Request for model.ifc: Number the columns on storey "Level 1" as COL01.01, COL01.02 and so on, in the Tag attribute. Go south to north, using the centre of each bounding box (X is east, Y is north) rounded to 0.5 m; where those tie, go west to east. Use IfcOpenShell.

First a look at what the model holds.

```python
import ifcopenshell
import ifcopenshell.util.element
import ifcopenshell.util.placement

model = ifcopenshell.open("model.ifc")
print(model.schema)
storey = next(s for s in model.by_type("IfcBuildingStorey") if s.Name == "Level 1")
columns = [e for e in ifcopenshell.util.element.get_decomposition(storey) if e.is_a("IfcColumn")]
for e in sorted(columns, key=lambda e: e.id()):
    origin = ifcopenshell.util.placement.get_local_placement(e.ObjectPlacement)[:3, 3]
    print(e.id(), e.Tag, e.Name, origin.round(2) + 0.0, sep=" | ")
```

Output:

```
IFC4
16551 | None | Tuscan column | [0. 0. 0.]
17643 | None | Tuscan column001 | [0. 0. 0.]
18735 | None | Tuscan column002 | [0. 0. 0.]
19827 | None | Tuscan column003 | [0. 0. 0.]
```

```python
import ifcopenshell
import ifcopenshell.geom
import ifcopenshell.util.element
import ifcopenshell.util.shape

model = ifcopenshell.open("model.ifc")
settings = ifcopenshell.geom.settings()
settings.set("use-world-coords", True)


def centre(element):
    shape = ifcopenshell.geom.create_shape(settings, element)
    return ifcopenshell.util.shape.get_bbox_centroid(shape.geometry)


storey = next(s for s in model.by_type("IfcBuildingStorey") if s.Name == "Level 1")
columns = [e for e in ifcopenshell.util.element.get_decomposition(storey) if e.is_a("IfcColumn")]

# Insertion points can sit at a corner or the storey origin, so sort by the geometry (in metres).
centres = {e: centre(e) for e in columns}
columns.sort(key=lambda e: (round(centres[e][1] / 0.5), centres[e][0]))

for i, e in enumerate(columns, start=1):
    number = f"COL01.{i:02d}"
    e.Tag = number
    print(e.id(), number)

model.write("model-out.ifc")
```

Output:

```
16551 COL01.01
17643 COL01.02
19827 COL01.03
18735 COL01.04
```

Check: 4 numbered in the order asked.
